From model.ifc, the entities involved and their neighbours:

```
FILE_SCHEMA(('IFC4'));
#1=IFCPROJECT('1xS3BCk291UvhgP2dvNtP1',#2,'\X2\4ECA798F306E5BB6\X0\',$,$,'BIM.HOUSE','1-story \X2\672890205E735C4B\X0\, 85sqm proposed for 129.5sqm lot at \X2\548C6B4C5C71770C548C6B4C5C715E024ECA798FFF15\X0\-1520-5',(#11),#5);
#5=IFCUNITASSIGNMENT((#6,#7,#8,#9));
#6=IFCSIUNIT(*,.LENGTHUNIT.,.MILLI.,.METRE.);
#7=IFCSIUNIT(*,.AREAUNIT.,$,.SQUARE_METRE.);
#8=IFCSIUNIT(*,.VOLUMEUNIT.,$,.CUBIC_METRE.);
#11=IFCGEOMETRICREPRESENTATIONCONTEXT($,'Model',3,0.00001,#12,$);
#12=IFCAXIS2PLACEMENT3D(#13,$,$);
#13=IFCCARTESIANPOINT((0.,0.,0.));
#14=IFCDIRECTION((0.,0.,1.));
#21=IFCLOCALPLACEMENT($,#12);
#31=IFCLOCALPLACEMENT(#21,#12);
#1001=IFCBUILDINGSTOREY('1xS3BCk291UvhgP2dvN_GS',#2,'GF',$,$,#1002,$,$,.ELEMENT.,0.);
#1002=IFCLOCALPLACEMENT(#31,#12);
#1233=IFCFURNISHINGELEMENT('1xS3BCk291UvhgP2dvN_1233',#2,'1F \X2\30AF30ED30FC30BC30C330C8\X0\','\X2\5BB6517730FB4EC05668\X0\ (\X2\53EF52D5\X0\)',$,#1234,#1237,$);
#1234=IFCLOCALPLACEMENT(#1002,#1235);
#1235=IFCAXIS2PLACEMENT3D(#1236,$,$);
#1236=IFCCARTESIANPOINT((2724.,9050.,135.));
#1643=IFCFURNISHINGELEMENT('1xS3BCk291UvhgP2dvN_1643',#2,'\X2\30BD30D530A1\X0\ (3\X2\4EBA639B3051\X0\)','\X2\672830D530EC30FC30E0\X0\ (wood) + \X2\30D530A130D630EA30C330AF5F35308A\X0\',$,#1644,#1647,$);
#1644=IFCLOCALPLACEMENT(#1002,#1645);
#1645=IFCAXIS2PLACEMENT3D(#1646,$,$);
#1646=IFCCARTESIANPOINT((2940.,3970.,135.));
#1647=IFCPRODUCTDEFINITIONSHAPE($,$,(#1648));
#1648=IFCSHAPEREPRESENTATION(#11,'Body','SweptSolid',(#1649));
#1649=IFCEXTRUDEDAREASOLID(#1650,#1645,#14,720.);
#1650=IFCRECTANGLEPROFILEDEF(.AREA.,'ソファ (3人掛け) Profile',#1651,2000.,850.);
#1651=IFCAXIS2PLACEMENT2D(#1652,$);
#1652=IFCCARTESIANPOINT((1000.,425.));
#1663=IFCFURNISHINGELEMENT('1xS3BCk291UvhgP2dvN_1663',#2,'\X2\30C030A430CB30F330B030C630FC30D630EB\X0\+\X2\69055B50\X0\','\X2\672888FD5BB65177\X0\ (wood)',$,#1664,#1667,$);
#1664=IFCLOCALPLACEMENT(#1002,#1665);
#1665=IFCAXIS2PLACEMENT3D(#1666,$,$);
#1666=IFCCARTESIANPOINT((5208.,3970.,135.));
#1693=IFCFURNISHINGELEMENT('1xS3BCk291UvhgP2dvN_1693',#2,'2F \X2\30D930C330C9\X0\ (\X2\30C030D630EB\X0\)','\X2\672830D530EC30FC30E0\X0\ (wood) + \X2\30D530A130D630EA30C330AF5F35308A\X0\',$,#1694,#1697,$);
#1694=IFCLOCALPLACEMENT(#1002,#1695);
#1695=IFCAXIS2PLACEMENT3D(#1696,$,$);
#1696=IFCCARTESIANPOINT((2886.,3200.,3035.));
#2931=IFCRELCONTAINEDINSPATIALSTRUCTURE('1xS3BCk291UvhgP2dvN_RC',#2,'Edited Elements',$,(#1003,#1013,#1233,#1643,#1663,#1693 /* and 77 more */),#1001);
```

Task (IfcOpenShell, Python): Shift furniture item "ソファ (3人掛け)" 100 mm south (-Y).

```python
import ifcopenshell
import ifcopenshell.api.geometry
import ifcopenshell.util.placement

model = ifcopenshell.open("model.ifc")

item = model.by_id(1643)
matrix = ifcopenshell.util.placement.get_local_placement(item.ObjectPlacement)
matrix[1, 3] -= 100.0
ifcopenshell.api.geometry.edit_object_placement(model, product=item, matrix=matrix, is_si=False)

print(ifcopenshell.util.placement.get_local_placement(item.ObjectPlacement).round(3) + 0.0)

model.write("model_v2.ifc")
```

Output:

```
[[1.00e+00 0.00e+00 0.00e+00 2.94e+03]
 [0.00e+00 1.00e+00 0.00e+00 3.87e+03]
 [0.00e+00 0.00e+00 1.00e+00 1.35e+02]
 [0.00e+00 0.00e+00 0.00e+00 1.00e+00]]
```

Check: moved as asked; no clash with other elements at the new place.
